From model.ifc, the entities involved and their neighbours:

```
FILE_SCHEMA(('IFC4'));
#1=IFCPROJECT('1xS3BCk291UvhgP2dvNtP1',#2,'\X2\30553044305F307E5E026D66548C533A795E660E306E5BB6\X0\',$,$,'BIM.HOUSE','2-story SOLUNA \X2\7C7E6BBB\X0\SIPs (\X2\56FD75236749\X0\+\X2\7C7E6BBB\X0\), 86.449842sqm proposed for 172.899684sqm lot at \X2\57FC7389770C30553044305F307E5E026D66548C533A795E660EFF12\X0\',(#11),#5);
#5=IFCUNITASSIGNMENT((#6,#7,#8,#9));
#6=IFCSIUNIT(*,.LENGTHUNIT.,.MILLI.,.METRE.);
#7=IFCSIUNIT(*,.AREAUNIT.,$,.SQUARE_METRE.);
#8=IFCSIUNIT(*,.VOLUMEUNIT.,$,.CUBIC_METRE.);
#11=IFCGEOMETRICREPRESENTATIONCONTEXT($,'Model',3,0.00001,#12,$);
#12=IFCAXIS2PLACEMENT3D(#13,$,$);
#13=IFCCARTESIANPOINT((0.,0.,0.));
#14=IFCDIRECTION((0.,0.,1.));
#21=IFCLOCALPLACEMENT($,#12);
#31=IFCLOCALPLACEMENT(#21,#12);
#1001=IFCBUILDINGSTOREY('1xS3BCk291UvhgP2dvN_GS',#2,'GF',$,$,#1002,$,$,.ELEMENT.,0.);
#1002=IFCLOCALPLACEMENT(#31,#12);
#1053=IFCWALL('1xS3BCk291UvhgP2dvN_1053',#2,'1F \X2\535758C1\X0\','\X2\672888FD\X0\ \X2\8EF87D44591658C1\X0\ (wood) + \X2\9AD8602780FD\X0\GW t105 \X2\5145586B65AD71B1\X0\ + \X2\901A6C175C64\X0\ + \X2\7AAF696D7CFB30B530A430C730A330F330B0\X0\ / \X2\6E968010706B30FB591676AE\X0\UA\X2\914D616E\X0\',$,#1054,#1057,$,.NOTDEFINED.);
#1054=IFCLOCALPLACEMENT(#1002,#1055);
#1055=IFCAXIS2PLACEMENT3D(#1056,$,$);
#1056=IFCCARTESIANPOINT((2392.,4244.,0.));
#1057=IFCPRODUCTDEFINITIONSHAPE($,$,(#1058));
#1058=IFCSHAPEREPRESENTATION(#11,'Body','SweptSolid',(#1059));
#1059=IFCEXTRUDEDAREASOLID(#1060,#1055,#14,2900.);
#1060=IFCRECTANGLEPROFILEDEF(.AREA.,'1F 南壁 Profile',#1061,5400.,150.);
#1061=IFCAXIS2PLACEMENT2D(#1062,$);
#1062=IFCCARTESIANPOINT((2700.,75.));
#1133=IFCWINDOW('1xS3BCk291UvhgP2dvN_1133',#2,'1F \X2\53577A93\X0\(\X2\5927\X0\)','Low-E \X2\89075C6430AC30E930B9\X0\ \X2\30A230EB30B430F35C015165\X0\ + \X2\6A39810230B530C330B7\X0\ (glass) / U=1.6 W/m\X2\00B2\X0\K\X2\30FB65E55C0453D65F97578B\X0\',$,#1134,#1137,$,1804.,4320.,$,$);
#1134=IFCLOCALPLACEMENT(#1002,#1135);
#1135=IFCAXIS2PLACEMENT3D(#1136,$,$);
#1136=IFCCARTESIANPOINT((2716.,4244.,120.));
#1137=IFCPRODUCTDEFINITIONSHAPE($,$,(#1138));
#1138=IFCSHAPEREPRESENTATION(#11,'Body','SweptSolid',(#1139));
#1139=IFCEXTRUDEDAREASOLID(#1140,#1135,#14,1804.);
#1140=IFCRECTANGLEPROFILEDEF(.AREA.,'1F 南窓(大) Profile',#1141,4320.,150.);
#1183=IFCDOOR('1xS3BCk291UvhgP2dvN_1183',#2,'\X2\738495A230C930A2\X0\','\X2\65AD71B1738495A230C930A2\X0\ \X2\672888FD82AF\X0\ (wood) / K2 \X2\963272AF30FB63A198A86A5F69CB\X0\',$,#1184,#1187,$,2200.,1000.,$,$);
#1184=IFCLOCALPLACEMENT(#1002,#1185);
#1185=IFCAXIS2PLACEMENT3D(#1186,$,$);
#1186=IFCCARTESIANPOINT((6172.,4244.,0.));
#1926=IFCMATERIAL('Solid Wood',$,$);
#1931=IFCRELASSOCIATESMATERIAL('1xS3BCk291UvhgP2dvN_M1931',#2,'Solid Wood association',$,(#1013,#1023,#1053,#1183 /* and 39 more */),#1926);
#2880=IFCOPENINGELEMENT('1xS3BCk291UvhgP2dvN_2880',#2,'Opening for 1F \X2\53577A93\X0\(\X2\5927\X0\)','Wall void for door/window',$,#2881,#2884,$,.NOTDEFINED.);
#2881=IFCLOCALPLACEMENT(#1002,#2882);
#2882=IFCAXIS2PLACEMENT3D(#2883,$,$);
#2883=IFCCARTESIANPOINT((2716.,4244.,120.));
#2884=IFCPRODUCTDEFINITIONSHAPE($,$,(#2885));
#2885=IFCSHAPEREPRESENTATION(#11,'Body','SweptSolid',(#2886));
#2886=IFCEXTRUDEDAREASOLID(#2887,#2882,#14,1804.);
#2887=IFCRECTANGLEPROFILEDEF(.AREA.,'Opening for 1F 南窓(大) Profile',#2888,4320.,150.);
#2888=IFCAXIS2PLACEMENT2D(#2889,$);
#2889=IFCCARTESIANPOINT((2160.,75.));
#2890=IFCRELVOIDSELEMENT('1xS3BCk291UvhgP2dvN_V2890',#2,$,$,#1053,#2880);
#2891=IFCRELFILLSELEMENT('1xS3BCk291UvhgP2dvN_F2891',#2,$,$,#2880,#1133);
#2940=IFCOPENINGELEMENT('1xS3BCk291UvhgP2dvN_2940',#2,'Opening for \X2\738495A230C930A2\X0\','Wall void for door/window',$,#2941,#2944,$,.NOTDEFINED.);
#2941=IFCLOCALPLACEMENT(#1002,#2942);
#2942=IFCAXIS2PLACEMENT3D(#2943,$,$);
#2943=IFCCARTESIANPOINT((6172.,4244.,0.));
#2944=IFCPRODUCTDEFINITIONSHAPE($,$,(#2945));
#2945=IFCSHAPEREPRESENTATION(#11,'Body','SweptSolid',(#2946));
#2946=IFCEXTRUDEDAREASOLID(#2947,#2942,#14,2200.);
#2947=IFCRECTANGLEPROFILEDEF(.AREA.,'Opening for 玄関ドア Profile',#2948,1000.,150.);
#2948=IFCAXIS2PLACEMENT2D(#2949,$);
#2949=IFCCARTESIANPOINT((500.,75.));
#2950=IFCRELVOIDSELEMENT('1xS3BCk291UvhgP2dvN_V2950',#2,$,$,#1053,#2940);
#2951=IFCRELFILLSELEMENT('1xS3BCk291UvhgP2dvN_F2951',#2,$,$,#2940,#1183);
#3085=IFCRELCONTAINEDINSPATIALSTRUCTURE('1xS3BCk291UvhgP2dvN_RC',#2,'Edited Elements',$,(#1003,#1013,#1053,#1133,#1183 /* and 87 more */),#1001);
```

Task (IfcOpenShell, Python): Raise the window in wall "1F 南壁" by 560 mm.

```python
import numpy as np
import ifcopenshell
import ifcopenshell.api.geometry
import ifcopenshell.util.placement
import ifcopenshell.util.unit

model = ifcopenshell.open("model.ifc")
unit_scale = ifcopenshell.util.unit.calculate_unit_scale(model)

window = model.by_guid("1xS3BCk291UvhgP2dvN_1133")
opening = window.FillsVoids[0].RelatingOpeningElement
dz = 0.56 / unit_scale

shift = np.array([0.0, 0.0, dz])
# The window is not placed relative to its opening, so move both.
for product in (opening, window):
    matrix = ifcopenshell.util.placement.get_local_placement(product.ObjectPlacement)
    matrix[:3, 3] += shift
    ifcopenshell.api.geometry.edit_object_placement(model, product=product, matrix=matrix, is_si=False)

print(f"moved by {dz * unit_scale:+.3f} m")

model.write("model_v2.ifc")
```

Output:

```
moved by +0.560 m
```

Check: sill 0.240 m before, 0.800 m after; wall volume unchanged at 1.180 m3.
